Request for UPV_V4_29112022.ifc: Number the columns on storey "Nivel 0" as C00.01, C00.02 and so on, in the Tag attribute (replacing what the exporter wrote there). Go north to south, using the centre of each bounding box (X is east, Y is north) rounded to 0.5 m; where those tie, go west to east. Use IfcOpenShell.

First a look at what the model holds.

```python
import ifcopenshell
import ifcopenshell.util.element
import ifcopenshell.util.placement

model = ifcopenshell.open("UPV_V4_29112022.ifc")
print(model.schema)
storey = next(s for s in model.by_type("IfcBuildingStorey") if s.Name == "Nivel 0")
columns = [e for e in ifcopenshell.util.element.get_decomposition(storey) if e.is_a("IfcColumn")]
for e in sorted(columns, key=lambda e: e.id()):
    origin = ifcopenshell.util.placement.get_local_placement(e.ObjectPlacement)[:3, 3]
    print(e.id(), e.Tag, e.Name, origin.round(2) + 0.0, sep=" | ")
```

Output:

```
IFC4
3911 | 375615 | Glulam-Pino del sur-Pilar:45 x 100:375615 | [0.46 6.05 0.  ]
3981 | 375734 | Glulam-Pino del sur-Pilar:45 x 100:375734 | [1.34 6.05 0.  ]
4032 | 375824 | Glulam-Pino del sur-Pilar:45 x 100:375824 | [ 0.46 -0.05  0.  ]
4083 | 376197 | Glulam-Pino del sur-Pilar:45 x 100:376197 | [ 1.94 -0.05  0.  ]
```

```python
import ifcopenshell
import ifcopenshell.geom
import ifcopenshell.util.element
import ifcopenshell.util.shape

model = ifcopenshell.open("UPV_V4_29112022.ifc")
settings = ifcopenshell.geom.settings()
settings.set("use-world-coords", True)


def centre(element):
    shape = ifcopenshell.geom.create_shape(settings, element)
    return ifcopenshell.util.shape.get_bbox_centroid(shape.geometry)


storey = next(s for s in model.by_type("IfcBuildingStorey") if s.Name == "Nivel 0")
columns = [e for e in ifcopenshell.util.element.get_decomposition(storey) if e.is_a("IfcColumn")]

# Insertion points can sit at a corner or the storey origin, so sort by the geometry (in metres).
centres = {e: centre(e) for e in columns}
columns.sort(key=lambda e: (-round(centres[e][1] / 0.5), centres[e][0]))

for i, e in enumerate(columns, start=1):
    number = f"C00.{i:02d}"
    e.Tag = number
    print(e.id(), number)

model.write("UPV_V4_29112022_rev.ifc")
```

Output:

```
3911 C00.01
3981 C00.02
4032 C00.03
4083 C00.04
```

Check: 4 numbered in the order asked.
